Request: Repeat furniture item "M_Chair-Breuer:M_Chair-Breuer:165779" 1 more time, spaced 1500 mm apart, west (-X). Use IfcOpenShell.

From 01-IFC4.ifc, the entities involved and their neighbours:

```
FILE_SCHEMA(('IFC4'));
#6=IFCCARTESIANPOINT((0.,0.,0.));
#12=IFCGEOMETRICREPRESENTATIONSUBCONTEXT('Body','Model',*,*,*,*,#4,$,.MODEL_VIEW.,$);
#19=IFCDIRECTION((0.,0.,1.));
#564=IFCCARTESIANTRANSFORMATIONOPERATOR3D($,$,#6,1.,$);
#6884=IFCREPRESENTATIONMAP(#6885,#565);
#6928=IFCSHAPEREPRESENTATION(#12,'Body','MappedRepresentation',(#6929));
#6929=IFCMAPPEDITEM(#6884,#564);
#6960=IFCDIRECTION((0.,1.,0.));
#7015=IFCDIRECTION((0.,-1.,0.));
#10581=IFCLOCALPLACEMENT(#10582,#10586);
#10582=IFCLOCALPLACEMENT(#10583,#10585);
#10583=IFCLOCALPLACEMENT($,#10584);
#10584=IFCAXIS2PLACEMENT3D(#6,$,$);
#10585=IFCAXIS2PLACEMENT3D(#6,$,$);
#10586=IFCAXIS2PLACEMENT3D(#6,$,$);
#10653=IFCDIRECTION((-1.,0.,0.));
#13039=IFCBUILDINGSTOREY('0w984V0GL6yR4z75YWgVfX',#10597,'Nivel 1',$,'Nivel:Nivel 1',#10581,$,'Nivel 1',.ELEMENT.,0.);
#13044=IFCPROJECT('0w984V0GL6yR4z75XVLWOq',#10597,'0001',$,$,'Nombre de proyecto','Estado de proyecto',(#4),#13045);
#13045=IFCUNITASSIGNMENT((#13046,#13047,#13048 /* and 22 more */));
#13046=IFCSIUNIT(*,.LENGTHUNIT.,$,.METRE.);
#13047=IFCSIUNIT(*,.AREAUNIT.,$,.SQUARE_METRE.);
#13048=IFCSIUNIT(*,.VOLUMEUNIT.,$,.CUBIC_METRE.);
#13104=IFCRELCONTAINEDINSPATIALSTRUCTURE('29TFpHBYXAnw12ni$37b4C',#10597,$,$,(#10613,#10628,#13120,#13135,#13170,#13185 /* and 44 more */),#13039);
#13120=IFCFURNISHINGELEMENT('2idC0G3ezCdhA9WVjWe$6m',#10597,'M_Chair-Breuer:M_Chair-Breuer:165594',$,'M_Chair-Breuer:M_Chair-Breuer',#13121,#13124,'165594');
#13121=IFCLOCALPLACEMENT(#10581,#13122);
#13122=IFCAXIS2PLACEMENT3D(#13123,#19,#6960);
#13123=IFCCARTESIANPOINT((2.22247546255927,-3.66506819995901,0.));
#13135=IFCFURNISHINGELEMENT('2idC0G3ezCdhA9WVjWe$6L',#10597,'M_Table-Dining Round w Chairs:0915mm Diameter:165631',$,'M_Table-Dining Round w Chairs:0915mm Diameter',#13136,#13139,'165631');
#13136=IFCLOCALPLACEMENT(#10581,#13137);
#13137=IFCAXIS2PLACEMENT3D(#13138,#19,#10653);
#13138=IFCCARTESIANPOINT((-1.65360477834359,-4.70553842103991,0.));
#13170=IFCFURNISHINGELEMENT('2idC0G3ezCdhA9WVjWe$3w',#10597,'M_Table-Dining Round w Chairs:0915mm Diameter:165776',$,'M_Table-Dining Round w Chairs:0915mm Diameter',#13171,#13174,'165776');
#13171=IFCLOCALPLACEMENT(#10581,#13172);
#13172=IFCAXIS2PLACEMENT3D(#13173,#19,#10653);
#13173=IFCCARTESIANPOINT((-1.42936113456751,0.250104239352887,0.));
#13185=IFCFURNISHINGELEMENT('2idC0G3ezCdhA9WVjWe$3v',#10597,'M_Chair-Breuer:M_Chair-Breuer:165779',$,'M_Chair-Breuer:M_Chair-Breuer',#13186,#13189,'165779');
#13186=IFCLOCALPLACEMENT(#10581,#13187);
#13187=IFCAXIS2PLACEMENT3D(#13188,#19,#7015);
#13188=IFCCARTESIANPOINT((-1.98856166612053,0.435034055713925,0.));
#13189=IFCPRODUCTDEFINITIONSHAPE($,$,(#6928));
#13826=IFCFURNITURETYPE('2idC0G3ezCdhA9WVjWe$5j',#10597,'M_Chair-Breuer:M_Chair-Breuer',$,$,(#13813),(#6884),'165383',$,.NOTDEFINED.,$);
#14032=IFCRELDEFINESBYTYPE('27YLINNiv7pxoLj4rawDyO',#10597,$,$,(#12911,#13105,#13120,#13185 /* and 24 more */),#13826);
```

```python
import numpy as np
import ifcopenshell
import ifcopenshell.api.geometry
import ifcopenshell.api.root
import ifcopenshell.util.element
import ifcopenshell.util.placement
import ifcopenshell.util.unit

model = ifcopenshell.open("01-IFC4.ifc")
unit_scale = ifcopenshell.util.unit.calculate_unit_scale(model)


def reuse_history(source, copy):
    """copy_class also copies each property set's owner history, people and application; keep the originals."""
    for rel in copy.IsDefinedBy:
        if rel.is_a("IfcRelDefinesByProperties") and (history := rel.RelatingPropertyDefinition.OwnerHistory):
            rel.RelatingPropertyDefinition.OwnerHistory = source.OwnerHistory
            ifcopenshell.util.element.remove_deep2(model, history)


source = model.by_id(13185)
base = ifcopenshell.util.placement.get_local_placement(source.ObjectPlacement)
step = np.array([-1.0, 0.0, 0.0]) * 1.5 / unit_scale

for i in range(1, 2):
    copy = ifcopenshell.api.root.copy_class(model, product=source)
    copy.Representation = ifcopenshell.util.element.copy_deep(
        model, source.Representation, exclude=["IfcGeometricRepresentationContext", "IfcRepresentationMap"]
    )
    copy.Name = "M_Chair-Breuer:M_Chair-Breuer"
    copy.Tag = None
    reuse_history(source, copy)
    matrix = base.copy()
    matrix[:3, 3] += i * step
    print("added at", matrix[:3, 3].round(3) + 0.0)
    ifcopenshell.api.geometry.edit_object_placement(model, product=copy, matrix=matrix, is_si=False)

model.write("01-IFC4-out.ifc")
```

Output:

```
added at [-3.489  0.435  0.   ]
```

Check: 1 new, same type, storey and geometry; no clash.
